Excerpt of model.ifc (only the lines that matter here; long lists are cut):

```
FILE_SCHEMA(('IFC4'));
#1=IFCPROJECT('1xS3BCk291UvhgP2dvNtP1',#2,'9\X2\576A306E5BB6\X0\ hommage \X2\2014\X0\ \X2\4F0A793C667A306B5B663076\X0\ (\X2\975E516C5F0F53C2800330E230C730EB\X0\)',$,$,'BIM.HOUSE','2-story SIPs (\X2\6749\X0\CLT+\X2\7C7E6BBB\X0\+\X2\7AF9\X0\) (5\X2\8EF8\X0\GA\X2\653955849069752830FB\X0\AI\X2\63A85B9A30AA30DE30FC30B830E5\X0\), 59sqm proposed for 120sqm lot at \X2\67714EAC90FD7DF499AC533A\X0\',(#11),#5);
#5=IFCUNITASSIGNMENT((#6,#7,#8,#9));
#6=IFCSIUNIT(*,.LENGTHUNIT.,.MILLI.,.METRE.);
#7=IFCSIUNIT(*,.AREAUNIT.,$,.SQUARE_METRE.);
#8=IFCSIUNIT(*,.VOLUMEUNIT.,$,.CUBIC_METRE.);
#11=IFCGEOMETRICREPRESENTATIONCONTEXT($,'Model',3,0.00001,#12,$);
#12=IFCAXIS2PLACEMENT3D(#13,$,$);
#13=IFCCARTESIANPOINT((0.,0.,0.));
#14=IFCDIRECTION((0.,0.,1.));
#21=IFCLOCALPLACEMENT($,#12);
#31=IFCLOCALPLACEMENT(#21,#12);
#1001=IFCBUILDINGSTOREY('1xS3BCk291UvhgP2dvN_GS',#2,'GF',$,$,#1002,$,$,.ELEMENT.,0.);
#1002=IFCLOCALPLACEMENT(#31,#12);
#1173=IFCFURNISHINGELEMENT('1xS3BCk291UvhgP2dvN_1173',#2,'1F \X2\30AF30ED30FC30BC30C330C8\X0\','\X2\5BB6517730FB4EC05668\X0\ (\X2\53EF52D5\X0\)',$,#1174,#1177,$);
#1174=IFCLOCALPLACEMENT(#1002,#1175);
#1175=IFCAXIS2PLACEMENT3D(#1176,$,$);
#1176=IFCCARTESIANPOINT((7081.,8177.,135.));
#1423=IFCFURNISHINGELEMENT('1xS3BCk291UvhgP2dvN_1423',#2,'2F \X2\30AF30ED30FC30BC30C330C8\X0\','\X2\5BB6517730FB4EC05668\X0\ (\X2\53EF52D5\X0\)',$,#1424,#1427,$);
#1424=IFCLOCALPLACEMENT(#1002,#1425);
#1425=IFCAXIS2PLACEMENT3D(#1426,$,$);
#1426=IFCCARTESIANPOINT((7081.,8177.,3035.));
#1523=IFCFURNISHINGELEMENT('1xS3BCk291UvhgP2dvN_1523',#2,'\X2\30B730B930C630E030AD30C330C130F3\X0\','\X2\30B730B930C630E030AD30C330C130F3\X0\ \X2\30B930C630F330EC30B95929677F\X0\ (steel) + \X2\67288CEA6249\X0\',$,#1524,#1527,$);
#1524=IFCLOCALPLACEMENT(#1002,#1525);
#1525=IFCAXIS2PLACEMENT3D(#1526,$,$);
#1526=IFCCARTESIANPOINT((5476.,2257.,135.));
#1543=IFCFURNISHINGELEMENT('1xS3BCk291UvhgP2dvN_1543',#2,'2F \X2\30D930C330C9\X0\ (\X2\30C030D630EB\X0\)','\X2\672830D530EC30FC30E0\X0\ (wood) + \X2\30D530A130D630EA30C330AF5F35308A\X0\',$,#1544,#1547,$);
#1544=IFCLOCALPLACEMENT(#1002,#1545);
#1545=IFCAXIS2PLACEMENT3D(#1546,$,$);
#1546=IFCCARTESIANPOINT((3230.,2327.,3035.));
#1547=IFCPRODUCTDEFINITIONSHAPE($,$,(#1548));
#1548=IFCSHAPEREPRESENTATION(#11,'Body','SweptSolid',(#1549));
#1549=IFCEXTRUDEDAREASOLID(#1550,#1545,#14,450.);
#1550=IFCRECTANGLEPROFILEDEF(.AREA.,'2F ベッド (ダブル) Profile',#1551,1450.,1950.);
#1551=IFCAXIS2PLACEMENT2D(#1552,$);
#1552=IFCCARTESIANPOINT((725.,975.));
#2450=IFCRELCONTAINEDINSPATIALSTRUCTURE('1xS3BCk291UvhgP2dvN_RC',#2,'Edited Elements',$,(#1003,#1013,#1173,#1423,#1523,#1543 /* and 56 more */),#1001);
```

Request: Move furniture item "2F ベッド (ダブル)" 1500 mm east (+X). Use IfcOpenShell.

```python
import ifcopenshell
import ifcopenshell.api.geometry
import ifcopenshell.util.placement
import ifcopenshell.util.unit

model = ifcopenshell.open("model.ifc")
unit_scale = ifcopenshell.util.unit.calculate_unit_scale(model)

item = model.by_id(1543)
matrix = ifcopenshell.util.placement.get_local_placement(item.ObjectPlacement)
matrix[0, 3] += 1.5 / unit_scale
ifcopenshell.api.geometry.edit_object_placement(model, product=item, matrix=matrix, is_si=False)

print(ifcopenshell.util.placement.get_local_placement(item.ObjectPlacement).round(3) + 0.0)

model.write("model_updated.ifc")
```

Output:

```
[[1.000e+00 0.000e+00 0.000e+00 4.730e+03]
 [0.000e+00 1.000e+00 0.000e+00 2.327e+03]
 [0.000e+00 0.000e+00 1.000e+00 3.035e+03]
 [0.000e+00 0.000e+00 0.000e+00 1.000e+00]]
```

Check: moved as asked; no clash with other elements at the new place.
